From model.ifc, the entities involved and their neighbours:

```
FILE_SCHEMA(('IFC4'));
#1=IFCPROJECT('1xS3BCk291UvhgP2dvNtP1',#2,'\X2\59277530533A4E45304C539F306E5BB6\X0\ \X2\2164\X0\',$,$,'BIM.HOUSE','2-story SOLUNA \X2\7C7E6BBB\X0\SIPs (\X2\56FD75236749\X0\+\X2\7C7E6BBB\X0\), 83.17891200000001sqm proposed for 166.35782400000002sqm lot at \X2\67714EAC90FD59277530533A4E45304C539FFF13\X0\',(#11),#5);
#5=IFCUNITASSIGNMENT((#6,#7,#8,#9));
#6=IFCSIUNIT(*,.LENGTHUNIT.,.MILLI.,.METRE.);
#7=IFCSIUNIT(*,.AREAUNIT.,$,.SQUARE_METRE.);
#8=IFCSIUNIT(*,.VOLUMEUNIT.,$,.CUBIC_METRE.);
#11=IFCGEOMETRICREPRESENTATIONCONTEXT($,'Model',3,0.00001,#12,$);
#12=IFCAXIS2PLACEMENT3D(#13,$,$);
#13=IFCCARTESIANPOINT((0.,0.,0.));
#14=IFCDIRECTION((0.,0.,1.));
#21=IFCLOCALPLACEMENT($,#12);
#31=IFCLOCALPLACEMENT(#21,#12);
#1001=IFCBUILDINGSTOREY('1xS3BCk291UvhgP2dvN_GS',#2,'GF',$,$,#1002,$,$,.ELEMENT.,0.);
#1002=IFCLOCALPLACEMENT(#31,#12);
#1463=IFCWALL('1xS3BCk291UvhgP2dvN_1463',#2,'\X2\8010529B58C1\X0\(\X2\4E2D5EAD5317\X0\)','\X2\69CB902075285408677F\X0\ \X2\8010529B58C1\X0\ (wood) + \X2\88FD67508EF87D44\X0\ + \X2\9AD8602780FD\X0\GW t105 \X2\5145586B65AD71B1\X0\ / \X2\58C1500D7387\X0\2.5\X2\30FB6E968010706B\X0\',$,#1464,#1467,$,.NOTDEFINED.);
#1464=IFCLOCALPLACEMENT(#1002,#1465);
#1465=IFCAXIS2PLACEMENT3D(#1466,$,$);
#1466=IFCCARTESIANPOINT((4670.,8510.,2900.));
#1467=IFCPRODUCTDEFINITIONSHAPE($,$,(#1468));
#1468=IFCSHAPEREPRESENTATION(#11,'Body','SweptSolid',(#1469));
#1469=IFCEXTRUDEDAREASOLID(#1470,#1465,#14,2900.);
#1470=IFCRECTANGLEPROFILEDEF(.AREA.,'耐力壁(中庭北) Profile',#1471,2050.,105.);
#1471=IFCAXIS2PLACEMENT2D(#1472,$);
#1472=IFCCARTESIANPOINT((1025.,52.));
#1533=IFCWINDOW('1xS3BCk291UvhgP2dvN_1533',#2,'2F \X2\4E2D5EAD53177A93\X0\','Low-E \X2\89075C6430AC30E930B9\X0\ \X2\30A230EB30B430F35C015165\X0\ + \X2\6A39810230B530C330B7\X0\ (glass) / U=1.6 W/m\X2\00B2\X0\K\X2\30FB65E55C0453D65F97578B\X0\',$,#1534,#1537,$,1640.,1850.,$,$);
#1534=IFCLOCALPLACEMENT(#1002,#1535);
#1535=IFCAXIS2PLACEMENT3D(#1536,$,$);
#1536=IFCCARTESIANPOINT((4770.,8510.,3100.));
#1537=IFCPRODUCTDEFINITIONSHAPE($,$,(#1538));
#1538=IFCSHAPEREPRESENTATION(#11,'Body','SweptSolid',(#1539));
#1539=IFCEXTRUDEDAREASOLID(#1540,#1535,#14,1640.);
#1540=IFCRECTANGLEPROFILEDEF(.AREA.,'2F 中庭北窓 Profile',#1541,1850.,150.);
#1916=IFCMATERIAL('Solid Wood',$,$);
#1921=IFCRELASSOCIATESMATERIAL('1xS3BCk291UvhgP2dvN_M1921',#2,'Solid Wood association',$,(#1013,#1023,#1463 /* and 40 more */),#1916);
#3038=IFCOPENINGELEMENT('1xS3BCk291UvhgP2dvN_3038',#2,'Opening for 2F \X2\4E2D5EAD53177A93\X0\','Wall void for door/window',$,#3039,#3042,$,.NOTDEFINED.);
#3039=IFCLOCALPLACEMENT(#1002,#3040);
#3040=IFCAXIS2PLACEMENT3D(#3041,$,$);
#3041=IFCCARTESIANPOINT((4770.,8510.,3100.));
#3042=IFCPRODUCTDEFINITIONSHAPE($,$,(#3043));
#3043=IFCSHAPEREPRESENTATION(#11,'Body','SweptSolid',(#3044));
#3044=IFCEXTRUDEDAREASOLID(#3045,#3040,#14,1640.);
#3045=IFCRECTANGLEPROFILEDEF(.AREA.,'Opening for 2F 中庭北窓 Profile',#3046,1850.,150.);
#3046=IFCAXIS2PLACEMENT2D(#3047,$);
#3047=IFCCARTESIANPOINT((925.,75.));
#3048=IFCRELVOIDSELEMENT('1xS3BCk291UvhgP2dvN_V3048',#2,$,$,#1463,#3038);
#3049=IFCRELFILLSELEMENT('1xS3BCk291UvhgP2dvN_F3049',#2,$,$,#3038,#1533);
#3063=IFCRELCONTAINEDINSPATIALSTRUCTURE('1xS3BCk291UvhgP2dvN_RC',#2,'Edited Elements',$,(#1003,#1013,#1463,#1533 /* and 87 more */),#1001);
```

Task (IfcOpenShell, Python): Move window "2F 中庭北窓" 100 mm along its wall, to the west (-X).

```python
import ifcopenshell
import ifcopenshell.api.geometry
import ifcopenshell.util.placement
import ifcopenshell.util.unit

model = ifcopenshell.open("model.ifc")
unit_scale = ifcopenshell.util.unit.calculate_unit_scale(model)

window = model.by_guid("1xS3BCk291UvhgP2dvN_1533")
opening = window.FillsVoids[0].RelatingOpeningElement
wall = opening.VoidsElements[0].RelatingBuildingElement

wall_matrix = ifcopenshell.util.placement.get_local_placement(wall.ObjectPlacement)
shift = wall_matrix[:3, 0] * -0.1 / unit_scale
before = ifcopenshell.util.placement.get_local_placement(window.ObjectPlacement)[:3, 3].copy()

# The window is not placed relative to its opening, so move both.
for product in (opening, window):
    matrix = ifcopenshell.util.placement.get_local_placement(product.ObjectPlacement)
    matrix[:3, 3] += shift
    ifcopenshell.api.geometry.edit_object_placement(model, product=product, matrix=matrix, is_si=False)

after = ifcopenshell.util.placement.get_local_placement(window.ObjectPlacement)[:3, 3]
print("window moved by", (after - before).round(3) + 0.0)

model.write("model_updated.ifc")
```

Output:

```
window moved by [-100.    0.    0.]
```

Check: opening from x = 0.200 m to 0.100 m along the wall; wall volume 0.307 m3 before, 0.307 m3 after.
